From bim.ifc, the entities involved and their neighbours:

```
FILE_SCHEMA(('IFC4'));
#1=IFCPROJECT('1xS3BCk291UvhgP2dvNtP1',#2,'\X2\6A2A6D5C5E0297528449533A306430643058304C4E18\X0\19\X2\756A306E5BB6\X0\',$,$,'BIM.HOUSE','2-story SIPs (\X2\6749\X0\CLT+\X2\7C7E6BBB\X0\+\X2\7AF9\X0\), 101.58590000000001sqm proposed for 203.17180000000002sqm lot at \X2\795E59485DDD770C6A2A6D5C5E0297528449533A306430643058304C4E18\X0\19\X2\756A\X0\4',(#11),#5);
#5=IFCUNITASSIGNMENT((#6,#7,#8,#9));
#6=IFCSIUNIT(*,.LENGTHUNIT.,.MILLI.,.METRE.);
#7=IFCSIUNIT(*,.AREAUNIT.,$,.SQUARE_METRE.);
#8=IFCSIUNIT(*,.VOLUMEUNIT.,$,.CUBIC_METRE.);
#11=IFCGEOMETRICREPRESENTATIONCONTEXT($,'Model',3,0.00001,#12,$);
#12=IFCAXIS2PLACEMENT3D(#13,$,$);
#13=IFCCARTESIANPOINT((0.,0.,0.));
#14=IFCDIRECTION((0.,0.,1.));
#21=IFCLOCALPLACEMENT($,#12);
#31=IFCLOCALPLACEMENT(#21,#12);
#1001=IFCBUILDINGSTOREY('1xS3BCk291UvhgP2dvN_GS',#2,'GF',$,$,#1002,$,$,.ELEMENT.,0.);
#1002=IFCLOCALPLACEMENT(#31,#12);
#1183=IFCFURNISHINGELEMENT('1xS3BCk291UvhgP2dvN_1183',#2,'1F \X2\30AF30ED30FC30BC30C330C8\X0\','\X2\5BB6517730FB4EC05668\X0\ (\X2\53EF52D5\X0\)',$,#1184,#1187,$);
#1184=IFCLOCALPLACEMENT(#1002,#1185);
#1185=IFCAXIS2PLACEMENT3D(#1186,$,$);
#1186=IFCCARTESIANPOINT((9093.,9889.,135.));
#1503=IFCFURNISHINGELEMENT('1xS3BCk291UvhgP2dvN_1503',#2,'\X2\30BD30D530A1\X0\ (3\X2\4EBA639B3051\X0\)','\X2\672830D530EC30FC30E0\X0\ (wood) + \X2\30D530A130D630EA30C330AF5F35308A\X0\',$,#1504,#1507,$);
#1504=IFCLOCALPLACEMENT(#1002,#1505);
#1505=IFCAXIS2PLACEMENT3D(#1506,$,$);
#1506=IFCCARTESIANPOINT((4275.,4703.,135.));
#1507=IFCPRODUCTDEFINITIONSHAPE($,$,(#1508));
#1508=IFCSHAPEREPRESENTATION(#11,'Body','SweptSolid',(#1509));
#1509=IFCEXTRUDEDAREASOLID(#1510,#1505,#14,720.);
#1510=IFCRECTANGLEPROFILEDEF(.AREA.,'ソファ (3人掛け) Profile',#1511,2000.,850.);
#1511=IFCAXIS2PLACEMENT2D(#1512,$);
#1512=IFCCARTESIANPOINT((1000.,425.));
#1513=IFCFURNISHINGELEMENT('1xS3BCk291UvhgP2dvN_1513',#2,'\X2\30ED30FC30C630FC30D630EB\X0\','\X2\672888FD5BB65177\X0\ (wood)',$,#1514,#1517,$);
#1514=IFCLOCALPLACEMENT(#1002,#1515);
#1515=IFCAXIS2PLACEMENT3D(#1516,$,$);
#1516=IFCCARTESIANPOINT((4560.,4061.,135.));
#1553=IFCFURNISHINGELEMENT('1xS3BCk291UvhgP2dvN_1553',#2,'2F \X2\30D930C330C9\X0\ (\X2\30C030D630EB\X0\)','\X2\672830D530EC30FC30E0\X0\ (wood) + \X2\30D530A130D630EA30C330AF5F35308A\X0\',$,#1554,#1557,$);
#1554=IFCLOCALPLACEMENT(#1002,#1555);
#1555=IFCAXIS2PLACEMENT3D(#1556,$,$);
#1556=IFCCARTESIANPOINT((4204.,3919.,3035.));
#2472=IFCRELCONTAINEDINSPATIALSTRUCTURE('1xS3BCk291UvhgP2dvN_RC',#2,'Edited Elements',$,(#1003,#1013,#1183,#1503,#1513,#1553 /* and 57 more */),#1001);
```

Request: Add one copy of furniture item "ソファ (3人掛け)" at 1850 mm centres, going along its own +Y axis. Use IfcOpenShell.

```python
import ifcopenshell
import ifcopenshell.api.geometry
import ifcopenshell.api.root
import ifcopenshell.util.element
import ifcopenshell.util.placement
import ifcopenshell.util.unit

model = ifcopenshell.open("bim.ifc")
unit_scale = ifcopenshell.util.unit.calculate_unit_scale(model)


def reuse_history(source, copy):
    """copy_class also copies each property set's owner history, people and application; keep the originals."""
    for rel in copy.IsDefinedBy:
        if rel.is_a("IfcRelDefinesByProperties") and (history := rel.RelatingPropertyDefinition.OwnerHistory):
            rel.RelatingPropertyDefinition.OwnerHistory = source.OwnerHistory
            ifcopenshell.util.element.remove_deep2(model, history)


source = model.by_guid("1xS3BCk291UvhgP2dvN_1503")
base = ifcopenshell.util.placement.get_local_placement(source.ObjectPlacement)
step = base[:3, 1] * 1.85 / unit_scale

for i in range(1, 2):
    copy = ifcopenshell.api.root.copy_class(model, product=source)
    copy.Representation = ifcopenshell.util.element.copy_deep(
        model, source.Representation, exclude=["IfcGeometricRepresentationContext", "IfcRepresentationMap"]
    )
    reuse_history(source, copy)
    matrix = base.copy()
    matrix[:3, 3] += i * step
    print("added at", matrix[:3, 3].round(3) + 0.0)
    ifcopenshell.api.geometry.edit_object_placement(model, product=copy, matrix=matrix, is_si=False)

model.write("bim-out.ifc")
```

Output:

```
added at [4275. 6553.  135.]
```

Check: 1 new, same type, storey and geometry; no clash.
